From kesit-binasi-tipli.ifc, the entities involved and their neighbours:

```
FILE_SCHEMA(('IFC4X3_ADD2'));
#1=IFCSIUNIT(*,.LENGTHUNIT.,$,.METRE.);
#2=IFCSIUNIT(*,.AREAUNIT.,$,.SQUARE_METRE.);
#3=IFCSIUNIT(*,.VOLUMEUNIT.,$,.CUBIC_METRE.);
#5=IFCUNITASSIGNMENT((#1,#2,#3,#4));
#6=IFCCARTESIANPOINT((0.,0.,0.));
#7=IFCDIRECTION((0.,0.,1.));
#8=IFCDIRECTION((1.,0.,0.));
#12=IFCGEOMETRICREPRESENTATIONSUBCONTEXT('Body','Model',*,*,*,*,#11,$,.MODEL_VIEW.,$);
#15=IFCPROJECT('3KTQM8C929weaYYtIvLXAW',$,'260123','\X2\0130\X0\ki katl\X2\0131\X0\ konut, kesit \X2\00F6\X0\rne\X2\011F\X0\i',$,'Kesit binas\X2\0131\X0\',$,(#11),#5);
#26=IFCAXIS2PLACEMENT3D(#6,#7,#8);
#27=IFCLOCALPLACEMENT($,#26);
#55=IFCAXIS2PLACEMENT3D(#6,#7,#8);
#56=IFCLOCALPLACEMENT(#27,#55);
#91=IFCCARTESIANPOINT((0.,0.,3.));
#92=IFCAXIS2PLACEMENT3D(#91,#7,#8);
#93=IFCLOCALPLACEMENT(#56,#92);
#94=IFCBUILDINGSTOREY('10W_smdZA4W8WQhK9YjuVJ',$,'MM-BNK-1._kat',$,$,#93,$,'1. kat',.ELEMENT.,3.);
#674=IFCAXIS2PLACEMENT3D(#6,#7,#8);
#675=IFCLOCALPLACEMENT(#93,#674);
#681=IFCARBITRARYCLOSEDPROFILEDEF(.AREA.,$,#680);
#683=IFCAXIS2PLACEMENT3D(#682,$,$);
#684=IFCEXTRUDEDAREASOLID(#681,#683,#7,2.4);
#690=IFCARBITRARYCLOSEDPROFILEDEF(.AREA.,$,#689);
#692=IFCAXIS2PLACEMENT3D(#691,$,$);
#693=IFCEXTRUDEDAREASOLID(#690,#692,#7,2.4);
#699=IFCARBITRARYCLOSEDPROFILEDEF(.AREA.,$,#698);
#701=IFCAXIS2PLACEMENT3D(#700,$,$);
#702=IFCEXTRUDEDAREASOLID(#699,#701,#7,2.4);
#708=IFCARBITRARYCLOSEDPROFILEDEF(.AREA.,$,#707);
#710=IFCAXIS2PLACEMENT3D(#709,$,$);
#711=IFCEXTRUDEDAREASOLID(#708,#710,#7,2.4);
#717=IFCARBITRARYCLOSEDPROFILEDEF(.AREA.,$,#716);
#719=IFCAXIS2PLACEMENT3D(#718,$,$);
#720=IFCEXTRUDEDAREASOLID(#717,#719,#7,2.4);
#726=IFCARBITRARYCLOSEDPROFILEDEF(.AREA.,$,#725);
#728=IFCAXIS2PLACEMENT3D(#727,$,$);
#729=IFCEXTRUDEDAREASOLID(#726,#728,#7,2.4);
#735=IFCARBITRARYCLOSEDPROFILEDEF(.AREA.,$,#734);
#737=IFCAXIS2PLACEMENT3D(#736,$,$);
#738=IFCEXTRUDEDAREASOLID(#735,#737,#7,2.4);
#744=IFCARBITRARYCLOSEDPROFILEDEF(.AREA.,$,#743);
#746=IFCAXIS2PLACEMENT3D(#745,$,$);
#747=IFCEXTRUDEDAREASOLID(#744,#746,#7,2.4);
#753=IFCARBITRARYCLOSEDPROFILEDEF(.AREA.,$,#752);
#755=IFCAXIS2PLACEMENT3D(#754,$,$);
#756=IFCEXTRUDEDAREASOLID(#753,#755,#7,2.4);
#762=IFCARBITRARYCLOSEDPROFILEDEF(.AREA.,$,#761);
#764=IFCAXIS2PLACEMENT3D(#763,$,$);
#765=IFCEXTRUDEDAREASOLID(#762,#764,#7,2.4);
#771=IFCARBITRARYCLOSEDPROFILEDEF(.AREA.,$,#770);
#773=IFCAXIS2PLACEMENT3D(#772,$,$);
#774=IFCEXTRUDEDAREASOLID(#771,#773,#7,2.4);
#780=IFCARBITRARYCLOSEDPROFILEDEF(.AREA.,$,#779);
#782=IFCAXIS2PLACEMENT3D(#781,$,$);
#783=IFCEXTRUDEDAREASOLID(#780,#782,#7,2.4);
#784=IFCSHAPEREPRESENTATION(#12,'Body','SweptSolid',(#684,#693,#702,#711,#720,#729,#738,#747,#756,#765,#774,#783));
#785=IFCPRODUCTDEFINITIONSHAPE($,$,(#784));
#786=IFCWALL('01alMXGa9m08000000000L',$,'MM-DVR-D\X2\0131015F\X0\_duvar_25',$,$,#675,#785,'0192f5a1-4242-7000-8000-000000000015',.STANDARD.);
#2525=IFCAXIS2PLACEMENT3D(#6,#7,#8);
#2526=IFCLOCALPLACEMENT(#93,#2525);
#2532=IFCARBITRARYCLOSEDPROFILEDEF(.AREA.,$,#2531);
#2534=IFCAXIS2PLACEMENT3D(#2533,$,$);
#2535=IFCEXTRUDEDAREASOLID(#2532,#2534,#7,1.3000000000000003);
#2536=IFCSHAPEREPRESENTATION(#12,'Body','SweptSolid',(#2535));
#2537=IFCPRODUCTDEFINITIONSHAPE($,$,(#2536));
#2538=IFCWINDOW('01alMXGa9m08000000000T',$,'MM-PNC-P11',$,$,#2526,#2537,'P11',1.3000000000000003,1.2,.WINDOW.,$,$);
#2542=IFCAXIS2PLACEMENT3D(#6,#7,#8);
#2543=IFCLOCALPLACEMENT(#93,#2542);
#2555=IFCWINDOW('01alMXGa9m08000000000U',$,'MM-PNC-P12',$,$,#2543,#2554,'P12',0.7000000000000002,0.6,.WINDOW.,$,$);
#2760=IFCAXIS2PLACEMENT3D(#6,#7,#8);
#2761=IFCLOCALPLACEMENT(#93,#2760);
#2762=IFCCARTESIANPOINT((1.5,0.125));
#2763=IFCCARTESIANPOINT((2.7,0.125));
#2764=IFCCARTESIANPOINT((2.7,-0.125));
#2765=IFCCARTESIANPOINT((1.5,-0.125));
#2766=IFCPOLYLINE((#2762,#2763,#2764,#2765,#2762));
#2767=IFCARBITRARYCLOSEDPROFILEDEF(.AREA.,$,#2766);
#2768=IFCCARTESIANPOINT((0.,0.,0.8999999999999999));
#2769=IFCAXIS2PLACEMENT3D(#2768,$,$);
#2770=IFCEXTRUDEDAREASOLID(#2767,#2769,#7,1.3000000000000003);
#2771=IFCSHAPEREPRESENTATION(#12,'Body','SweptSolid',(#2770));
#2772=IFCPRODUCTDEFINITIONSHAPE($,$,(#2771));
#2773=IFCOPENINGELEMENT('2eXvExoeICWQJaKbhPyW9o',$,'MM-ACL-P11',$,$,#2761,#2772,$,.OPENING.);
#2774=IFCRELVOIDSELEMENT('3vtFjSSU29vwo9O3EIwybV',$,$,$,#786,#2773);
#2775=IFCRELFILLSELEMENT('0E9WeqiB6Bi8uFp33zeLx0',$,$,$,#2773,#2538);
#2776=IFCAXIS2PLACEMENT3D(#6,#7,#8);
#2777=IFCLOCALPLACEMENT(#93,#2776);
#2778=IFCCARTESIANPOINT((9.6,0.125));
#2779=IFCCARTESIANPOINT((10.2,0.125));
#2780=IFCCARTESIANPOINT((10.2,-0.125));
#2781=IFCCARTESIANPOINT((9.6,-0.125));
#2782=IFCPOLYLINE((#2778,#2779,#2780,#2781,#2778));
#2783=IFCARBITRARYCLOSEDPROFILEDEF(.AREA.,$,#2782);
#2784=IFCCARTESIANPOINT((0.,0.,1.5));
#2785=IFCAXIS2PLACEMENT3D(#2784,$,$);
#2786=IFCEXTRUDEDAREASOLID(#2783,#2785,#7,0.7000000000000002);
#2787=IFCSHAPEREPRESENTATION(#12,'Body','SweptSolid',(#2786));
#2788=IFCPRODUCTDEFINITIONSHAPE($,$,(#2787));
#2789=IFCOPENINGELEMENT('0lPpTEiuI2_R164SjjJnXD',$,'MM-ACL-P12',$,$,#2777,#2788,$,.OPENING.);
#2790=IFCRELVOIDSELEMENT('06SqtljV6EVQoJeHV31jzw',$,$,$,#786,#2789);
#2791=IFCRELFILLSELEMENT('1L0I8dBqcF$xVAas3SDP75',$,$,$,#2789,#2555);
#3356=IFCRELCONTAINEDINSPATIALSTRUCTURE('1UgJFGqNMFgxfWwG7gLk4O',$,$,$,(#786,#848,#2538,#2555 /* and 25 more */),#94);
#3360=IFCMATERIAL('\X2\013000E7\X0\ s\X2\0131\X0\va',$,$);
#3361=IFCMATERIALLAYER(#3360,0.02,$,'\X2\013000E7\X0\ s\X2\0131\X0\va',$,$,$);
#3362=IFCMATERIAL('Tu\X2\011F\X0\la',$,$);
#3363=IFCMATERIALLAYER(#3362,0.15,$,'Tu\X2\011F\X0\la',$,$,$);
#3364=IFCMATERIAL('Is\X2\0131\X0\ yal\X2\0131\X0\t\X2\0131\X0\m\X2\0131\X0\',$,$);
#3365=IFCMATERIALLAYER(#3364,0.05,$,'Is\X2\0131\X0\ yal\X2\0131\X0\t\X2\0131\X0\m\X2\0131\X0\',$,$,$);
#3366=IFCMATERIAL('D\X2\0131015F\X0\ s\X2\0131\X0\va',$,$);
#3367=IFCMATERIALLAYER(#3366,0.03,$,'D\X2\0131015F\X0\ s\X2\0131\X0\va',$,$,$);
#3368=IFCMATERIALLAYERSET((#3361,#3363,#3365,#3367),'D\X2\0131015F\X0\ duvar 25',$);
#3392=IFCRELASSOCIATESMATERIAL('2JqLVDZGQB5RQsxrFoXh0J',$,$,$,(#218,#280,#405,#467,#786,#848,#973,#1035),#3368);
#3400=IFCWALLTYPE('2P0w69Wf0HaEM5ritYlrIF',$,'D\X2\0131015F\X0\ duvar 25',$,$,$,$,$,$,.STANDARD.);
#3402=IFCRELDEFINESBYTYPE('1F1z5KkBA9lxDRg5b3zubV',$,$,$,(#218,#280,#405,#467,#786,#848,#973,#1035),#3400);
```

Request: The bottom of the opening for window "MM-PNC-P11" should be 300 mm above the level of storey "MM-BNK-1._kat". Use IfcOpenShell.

```python
import numpy as np
import ifcopenshell
import ifcopenshell.api.geometry
import ifcopenshell.geom
import ifcopenshell.util.element
import ifcopenshell.util.placement
import ifcopenshell.util.shape
import ifcopenshell.util.unit

model = ifcopenshell.open("kesit-binasi-tipli.ifc")
unit_scale = ifcopenshell.util.unit.calculate_unit_scale(model)

window = model.by_id(2538)
opening = window.FillsVoids[0].RelatingOpeningElement
storey = ifcopenshell.util.element.get_container(window, ifc_class="IfcBuildingStorey")
level = ifcopenshell.util.placement.get_local_placement(storey.ObjectPlacement)[2, 3]

# The opening's origin need not be at the sill, so measure its lowest point.
shape = ifcopenshell.geom.create_shape(ifcopenshell.geom.settings(), opening)
bottom = ifcopenshell.util.shape.get_shape_bottom_elevation(shape, shape.geometry) / unit_scale
dz = level + 0.3 / unit_scale - bottom

shift = np.array([0.0, 0.0, dz])
# The window is not placed relative to its opening, so move both.
for product in (opening, window):
    matrix = ifcopenshell.util.placement.get_local_placement(product.ObjectPlacement)
    matrix[:3, 3] += shift
    ifcopenshell.api.geometry.edit_object_placement(model, product=product, matrix=matrix, is_si=False)

print(f"moved by {dz * unit_scale:+.3f} m")

model.write("kesit-binasi-tipli_v2.ifc")
```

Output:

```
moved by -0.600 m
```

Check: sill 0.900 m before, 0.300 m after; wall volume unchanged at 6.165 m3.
